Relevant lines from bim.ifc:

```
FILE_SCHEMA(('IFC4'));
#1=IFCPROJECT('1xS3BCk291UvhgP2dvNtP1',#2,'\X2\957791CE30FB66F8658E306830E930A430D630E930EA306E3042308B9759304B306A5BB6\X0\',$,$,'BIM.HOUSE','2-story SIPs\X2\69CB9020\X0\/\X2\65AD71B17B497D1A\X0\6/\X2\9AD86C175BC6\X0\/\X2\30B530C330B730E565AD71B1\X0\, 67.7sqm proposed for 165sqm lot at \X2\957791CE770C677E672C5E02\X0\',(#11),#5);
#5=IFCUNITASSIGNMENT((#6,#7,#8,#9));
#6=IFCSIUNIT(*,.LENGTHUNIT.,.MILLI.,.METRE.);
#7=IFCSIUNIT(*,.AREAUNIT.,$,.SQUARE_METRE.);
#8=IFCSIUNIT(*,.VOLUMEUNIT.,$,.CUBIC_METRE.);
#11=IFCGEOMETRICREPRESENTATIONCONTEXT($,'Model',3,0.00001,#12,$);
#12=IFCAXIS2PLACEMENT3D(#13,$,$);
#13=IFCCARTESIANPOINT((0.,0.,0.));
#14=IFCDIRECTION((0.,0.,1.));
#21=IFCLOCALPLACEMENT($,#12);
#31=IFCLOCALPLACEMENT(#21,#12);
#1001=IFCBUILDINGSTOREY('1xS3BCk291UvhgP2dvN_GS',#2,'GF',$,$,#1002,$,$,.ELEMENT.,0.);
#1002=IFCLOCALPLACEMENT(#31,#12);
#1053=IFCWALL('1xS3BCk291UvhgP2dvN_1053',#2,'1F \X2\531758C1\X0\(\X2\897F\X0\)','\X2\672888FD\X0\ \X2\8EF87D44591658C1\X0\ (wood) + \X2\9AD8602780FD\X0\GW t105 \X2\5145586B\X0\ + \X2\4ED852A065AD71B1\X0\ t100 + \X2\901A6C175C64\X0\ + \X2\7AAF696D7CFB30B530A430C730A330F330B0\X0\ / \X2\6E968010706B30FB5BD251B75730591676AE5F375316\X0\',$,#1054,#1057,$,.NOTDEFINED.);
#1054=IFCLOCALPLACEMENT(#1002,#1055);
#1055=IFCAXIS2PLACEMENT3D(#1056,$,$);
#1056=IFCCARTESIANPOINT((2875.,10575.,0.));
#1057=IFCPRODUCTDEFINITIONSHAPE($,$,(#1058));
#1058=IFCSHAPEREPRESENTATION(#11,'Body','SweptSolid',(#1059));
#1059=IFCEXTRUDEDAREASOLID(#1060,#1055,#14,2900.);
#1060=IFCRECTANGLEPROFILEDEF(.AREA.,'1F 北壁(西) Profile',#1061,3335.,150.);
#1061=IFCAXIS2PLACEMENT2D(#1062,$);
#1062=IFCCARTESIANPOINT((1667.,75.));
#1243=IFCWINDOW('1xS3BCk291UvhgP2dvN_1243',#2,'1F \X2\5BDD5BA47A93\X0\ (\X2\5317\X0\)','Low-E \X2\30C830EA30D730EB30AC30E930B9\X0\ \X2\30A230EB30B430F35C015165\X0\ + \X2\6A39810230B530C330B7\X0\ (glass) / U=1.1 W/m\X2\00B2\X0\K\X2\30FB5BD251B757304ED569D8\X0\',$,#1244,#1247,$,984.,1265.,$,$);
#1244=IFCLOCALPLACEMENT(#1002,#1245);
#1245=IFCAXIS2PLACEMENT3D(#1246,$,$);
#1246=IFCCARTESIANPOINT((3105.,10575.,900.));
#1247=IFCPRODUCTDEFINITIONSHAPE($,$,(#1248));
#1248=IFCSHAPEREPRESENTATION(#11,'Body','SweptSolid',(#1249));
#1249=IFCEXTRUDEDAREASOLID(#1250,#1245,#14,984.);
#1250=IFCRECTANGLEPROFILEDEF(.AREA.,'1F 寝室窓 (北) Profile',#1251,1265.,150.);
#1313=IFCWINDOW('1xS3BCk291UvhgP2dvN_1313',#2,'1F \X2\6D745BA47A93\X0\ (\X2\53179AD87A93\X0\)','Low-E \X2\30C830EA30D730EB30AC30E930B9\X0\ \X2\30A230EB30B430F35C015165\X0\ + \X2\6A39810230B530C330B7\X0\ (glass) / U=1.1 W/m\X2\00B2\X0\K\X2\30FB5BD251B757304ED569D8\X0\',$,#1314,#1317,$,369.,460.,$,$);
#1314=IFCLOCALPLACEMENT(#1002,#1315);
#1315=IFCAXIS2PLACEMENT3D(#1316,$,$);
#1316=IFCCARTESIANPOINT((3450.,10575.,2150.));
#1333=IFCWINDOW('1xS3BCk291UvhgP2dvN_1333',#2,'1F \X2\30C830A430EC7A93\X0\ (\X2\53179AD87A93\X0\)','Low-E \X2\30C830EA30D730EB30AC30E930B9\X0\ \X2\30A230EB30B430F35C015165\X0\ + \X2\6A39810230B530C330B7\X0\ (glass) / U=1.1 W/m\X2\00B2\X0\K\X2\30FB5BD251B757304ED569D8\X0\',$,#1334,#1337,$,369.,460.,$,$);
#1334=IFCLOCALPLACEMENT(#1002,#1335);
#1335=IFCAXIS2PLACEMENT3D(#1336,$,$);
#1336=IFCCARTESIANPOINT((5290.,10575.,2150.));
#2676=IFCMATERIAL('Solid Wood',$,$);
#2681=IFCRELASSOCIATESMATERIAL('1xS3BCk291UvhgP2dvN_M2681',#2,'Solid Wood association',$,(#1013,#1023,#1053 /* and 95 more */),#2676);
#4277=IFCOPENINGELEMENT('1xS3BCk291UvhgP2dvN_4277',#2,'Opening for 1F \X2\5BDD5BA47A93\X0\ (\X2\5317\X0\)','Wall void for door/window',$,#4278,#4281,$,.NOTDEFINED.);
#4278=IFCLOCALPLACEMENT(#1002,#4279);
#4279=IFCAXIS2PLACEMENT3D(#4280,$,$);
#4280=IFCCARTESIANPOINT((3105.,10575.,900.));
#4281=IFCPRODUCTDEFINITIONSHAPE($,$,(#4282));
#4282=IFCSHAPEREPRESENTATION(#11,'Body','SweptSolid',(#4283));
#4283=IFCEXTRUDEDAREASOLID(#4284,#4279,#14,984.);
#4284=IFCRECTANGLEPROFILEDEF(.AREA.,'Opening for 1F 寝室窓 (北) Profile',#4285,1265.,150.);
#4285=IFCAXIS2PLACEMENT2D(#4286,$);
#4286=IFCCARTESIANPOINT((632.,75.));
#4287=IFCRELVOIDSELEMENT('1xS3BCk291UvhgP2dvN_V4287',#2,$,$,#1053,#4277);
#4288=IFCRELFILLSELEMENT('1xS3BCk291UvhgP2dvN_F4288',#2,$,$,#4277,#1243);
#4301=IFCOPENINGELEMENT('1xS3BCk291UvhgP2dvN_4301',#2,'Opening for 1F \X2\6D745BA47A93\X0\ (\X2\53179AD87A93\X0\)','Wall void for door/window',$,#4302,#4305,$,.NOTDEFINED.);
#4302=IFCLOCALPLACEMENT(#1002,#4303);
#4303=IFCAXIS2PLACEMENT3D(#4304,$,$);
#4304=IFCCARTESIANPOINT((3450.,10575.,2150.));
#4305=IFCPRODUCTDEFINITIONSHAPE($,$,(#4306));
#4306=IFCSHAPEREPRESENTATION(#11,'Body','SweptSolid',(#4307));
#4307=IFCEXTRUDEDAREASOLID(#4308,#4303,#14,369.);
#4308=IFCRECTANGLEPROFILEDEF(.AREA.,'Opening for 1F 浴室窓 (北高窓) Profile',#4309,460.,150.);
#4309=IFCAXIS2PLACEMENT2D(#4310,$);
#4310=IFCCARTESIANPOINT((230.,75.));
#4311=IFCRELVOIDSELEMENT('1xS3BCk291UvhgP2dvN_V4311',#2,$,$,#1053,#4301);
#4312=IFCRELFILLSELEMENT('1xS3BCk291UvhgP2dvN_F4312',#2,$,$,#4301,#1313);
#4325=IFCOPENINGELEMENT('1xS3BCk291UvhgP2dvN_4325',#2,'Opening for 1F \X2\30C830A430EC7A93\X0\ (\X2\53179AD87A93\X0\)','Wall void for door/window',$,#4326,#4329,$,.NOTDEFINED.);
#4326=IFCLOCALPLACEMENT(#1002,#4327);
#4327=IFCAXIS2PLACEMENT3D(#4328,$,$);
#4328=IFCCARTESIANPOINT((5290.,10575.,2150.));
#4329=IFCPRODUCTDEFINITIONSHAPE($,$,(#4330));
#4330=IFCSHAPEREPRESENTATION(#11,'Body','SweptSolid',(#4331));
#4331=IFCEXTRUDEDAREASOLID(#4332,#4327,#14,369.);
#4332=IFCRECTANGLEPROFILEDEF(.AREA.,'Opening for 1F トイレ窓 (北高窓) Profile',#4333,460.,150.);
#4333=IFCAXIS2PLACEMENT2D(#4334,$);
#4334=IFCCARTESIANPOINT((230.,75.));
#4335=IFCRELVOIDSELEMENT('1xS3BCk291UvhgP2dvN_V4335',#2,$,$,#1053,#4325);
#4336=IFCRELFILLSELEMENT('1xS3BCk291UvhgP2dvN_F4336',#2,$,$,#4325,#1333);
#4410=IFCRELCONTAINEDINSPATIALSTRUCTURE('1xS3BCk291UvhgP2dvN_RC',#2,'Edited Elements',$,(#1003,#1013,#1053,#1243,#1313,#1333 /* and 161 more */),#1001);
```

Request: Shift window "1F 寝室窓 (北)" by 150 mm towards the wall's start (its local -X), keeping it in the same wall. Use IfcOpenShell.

```python
import ifcopenshell
import ifcopenshell.api.geometry
import ifcopenshell.util.placement
import ifcopenshell.util.unit

model = ifcopenshell.open("bim.ifc")
unit_scale = ifcopenshell.util.unit.calculate_unit_scale(model)

window = model.by_id(1243)
opening = window.FillsVoids[0].RelatingOpeningElement
wall = opening.VoidsElements[0].RelatingBuildingElement

wall_matrix = ifcopenshell.util.placement.get_local_placement(wall.ObjectPlacement)
shift = wall_matrix[:3, 0] * -0.15 / unit_scale
before = ifcopenshell.util.placement.get_local_placement(window.ObjectPlacement)[:3, 3].copy()

# The window is not placed relative to its opening, so move both.
for product in (opening, window):
    matrix = ifcopenshell.util.placement.get_local_placement(product.ObjectPlacement)
    matrix[:3, 3] += shift
    ifcopenshell.api.geometry.edit_object_placement(model, product=product, matrix=matrix, is_si=False)

after = ifcopenshell.util.placement.get_local_placement(window.ObjectPlacement)[:3, 3]
print("window moved by", (after - before).round(3) + 0.0)

model.write("bim-out.ifc")
```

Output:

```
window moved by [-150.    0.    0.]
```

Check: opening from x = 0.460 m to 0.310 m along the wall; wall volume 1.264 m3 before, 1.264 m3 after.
